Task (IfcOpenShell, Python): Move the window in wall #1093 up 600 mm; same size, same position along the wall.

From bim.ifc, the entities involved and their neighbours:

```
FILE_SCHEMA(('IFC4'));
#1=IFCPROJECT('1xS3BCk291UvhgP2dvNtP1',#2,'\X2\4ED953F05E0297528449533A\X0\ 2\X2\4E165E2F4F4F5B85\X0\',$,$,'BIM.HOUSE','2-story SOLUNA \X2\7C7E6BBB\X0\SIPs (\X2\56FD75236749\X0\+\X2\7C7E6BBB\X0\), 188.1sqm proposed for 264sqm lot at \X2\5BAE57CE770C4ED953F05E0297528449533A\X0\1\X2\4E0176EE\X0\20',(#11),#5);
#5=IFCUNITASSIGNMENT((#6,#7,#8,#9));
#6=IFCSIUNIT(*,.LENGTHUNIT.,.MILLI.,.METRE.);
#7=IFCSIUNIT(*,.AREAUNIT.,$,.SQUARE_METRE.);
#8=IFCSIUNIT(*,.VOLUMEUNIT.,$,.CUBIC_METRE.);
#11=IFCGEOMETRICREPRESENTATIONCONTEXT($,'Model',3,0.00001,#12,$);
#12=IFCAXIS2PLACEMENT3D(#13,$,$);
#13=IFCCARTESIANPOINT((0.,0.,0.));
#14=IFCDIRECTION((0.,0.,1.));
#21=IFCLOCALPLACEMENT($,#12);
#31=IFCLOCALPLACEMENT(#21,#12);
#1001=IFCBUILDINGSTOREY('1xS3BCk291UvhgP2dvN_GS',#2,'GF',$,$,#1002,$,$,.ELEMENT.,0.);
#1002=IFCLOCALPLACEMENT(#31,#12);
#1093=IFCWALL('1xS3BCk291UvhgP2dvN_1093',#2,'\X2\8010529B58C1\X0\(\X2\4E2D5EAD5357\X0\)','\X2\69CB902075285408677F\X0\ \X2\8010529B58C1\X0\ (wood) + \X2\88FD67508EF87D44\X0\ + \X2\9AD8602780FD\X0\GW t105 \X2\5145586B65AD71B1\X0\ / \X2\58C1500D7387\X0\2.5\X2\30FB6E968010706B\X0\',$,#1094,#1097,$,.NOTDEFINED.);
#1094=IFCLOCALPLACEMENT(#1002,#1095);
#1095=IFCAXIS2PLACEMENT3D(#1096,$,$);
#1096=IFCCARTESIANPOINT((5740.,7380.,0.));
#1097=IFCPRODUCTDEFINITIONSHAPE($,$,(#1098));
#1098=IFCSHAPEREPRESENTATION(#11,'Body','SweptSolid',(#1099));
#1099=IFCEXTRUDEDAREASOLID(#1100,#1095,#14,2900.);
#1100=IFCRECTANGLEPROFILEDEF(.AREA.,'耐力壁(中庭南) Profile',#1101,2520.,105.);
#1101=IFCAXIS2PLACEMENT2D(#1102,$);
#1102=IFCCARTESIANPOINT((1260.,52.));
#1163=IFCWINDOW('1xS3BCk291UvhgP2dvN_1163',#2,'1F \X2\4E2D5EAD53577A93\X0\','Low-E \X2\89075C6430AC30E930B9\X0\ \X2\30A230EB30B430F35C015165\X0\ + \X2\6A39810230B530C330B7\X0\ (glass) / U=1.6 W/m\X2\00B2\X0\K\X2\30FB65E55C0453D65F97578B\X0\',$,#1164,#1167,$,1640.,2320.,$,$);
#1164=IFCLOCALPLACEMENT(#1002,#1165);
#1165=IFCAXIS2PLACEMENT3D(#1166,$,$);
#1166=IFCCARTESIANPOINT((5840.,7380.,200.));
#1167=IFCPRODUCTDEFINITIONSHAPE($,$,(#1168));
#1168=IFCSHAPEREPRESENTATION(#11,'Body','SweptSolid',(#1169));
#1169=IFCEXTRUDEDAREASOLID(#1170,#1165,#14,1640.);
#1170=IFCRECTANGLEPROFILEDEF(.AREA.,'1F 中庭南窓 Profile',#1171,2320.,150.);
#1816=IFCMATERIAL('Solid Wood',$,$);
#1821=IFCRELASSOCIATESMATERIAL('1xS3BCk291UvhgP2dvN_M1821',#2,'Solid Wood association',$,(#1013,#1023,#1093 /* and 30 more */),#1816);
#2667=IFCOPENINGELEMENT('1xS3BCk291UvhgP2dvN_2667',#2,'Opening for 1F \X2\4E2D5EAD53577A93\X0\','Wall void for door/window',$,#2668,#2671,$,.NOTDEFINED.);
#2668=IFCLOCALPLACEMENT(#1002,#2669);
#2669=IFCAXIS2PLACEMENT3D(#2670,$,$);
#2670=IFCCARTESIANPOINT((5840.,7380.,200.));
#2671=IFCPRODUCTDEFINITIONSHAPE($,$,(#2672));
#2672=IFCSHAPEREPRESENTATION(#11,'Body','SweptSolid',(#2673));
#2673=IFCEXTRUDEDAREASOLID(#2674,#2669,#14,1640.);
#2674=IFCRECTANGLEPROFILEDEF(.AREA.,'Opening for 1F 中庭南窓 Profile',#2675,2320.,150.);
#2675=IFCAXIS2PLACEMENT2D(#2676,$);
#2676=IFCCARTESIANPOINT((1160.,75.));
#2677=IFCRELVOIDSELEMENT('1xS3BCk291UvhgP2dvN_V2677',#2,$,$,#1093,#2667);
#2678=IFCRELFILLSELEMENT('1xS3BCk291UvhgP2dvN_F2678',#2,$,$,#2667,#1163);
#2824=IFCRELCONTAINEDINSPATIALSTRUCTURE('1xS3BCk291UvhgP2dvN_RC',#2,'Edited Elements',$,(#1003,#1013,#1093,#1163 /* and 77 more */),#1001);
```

```python
import numpy as np
import ifcopenshell
import ifcopenshell.api.geometry
import ifcopenshell.util.placement
import ifcopenshell.util.unit

model = ifcopenshell.open("bim.ifc")
unit_scale = ifcopenshell.util.unit.calculate_unit_scale(model)

window = model.by_guid("1xS3BCk291UvhgP2dvN_1163")
opening = window.FillsVoids[0].RelatingOpeningElement
dz = 0.6 / unit_scale

shift = np.array([0.0, 0.0, dz])
# The window is not placed relative to its opening, so move both.
for product in (opening, window):
    matrix = ifcopenshell.util.placement.get_local_placement(product.ObjectPlacement)
    matrix[:3, 3] += shift
    ifcopenshell.api.geometry.edit_object_placement(model, product=product, matrix=matrix, is_si=False)

print(f"moved by {dz * unit_scale:+.3f} m")

model.write("bim_rev.ifc")
```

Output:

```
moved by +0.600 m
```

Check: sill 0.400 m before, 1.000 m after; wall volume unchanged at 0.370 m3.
